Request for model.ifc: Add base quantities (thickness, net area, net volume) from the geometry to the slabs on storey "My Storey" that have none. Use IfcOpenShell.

First a look at what the model holds.

```python
import ifcopenshell
import ifcopenshell.util.element
import ifcopenshell.util.unit

model = ifcopenshell.open("model.ifc")
print(model.schema)
for unit_type in ("LENGTHUNIT", "AREAUNIT", "VOLUMEUNIT"):
    print(unit_type, ifcopenshell.util.unit.calculate_unit_scale(model, unit_type))
storey = next(s for s in model.by_type("IfcBuildingStorey") if s.Name == "My Storey")
slabs = [e for e in ifcopenshell.util.element.get_decomposition(storey) if e.is_a("IfcSlab")]
for e in sorted(slabs, key=lambda e: e.id()):
    print(e.id(), e.is_a(), e.Name, list(ifcopenshell.util.element.get_psets(e, qtos_only=True)), sep=" | ")
```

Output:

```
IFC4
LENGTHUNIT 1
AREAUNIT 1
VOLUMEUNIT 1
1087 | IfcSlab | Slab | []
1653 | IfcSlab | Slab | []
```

```python
import ifcopenshell
import ifcopenshell.api.pset
import ifcopenshell.geom
import ifcopenshell.util.element
import ifcopenshell.util.shape
import ifcopenshell.util.unit

model = ifcopenshell.open("model.ifc")
unit_scale = ifcopenshell.util.unit.calculate_unit_scale(model)
area_scale = ifcopenshell.util.unit.calculate_unit_scale(model, "AREAUNIT")
volume_scale = ifcopenshell.util.unit.calculate_unit_scale(model, "VOLUMEUNIT")
settings = ifcopenshell.geom.settings()

storey = next(s for s in model.by_type("IfcBuildingStorey") if s.Name == "My Storey")
slabs = [e for e in ifcopenshell.util.element.get_decomposition(storey) if e.is_a("IfcSlab")]

for e in sorted(slabs, key=lambda e: e.id()):
    if ifcopenshell.util.element.get_psets(e, qtos_only=True, should_inherit=False):
        continue
    # Geometry comes back in metres, in the element's own axes.
    shape = ifcopenshell.geom.create_shape(settings, e)
    values = {
        "Width": ifcopenshell.util.shape.get_z(shape.geometry) / unit_scale,
        "NetArea": ifcopenshell.util.shape.get_footprint_area(shape.geometry) / area_scale,
        "NetVolume": ifcopenshell.util.shape.get_volume(shape.geometry) / volume_scale,
    }
    qto = ifcopenshell.api.pset.add_qto(model, product=e, name="Qto_SlabBaseQuantities")
    ifcopenshell.api.pset.edit_qto(model, qto=qto, properties=values)
    print(e.id(), {k: round(v, 3) for k, v in values.items()})

model.write("model_rev.ifc")
```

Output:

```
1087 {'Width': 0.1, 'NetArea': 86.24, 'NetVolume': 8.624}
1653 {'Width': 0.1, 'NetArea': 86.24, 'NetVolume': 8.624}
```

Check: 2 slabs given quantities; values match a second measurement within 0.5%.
